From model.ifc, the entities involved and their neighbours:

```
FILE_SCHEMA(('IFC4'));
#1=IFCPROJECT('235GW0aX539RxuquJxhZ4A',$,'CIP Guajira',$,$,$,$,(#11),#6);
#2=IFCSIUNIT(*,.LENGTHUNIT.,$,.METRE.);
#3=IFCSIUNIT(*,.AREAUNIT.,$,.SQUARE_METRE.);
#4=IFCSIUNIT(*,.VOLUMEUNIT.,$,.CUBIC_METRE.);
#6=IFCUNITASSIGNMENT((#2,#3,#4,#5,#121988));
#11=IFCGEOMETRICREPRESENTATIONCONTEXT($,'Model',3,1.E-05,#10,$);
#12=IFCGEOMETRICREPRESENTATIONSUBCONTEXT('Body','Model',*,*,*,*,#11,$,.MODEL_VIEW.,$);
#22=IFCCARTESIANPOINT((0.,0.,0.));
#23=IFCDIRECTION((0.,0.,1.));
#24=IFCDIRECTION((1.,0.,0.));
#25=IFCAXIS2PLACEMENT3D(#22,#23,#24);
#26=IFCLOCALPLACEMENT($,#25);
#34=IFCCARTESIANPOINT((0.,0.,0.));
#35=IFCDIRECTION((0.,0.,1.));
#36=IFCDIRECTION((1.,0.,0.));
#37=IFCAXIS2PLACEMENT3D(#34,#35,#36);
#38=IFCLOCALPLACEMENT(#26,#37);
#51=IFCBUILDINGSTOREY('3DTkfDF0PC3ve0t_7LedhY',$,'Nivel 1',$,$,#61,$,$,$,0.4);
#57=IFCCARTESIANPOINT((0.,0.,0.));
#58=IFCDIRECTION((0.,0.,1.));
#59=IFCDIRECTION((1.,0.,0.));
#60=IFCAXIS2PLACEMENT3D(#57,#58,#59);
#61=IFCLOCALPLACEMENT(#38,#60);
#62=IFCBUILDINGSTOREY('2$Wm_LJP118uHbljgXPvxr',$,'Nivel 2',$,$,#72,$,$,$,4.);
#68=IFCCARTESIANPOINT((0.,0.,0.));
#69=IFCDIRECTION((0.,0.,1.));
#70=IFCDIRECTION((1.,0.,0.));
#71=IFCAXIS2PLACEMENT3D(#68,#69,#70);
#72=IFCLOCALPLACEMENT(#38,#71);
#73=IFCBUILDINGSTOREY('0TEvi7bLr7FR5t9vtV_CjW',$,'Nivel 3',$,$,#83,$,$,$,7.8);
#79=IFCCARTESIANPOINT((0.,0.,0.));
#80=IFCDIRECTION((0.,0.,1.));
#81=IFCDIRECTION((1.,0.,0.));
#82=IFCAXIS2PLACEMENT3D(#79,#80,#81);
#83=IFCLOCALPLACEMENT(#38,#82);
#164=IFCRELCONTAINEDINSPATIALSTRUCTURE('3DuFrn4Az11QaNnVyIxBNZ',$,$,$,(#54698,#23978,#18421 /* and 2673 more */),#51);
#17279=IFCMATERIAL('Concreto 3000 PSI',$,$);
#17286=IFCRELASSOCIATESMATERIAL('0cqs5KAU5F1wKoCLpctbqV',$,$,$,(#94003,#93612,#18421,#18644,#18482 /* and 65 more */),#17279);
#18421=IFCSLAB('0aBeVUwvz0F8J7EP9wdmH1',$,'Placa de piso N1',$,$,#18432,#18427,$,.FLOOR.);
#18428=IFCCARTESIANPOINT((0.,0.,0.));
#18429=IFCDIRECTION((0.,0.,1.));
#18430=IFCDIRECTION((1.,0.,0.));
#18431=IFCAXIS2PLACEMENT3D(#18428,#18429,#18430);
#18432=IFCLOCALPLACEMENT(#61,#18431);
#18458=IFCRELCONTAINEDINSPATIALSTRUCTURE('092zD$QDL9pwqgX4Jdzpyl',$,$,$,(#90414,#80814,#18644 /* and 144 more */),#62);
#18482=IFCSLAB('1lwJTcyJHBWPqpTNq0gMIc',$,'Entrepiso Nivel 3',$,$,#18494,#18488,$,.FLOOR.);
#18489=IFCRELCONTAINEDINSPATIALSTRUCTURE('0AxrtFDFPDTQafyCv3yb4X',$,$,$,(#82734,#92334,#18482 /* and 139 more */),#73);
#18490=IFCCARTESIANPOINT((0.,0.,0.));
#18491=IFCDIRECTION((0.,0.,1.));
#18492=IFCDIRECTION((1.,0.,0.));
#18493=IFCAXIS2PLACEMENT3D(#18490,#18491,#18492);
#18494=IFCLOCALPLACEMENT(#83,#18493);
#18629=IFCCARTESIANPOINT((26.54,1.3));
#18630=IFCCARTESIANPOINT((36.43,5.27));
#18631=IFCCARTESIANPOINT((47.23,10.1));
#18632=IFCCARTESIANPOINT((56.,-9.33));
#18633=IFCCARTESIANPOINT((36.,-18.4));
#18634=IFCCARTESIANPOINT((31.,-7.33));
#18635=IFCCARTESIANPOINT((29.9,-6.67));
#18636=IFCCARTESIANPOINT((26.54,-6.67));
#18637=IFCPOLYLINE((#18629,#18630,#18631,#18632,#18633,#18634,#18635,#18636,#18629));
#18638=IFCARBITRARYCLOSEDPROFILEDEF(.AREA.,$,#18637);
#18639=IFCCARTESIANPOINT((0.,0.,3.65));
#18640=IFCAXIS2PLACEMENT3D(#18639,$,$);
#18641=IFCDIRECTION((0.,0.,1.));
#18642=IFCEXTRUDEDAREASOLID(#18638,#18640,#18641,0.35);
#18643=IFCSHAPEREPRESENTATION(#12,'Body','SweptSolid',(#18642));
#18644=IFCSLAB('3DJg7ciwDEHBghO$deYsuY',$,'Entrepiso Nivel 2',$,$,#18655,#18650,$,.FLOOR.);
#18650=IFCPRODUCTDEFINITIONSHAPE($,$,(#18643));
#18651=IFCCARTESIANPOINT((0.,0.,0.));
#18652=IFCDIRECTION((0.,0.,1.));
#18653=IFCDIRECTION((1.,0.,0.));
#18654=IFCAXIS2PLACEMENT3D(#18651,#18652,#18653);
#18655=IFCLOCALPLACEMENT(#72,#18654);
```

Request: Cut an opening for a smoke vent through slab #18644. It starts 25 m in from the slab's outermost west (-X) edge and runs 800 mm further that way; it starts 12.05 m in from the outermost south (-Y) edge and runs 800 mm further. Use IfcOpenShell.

```python
import numpy as np
import ifcopenshell
import ifcopenshell.api.feature
import ifcopenshell.api.geometry
import ifcopenshell.api.root
import ifcopenshell.geom
import ifcopenshell.util.placement
import ifcopenshell.util.representation
import ifcopenshell.util.shape
import ifcopenshell.util.unit

model = ifcopenshell.open("model.ifc")
unit_scale = ifcopenshell.util.unit.calculate_unit_scale(model)
settings = ifcopenshell.geom.settings()


def volume(element):
    """Net volume in cubic metres, openings subtracted."""
    shape = ifcopenshell.geom.create_shape(settings, element)
    return ifcopenshell.util.shape.get_volume(shape.geometry)


slab = model.by_guid("3DJg7ciwDEHBghO$deYsuY")
before = volume(slab)

# Extent in the slab's own axes, in metres. The edges named are its -X and -Y sides.
slab_shape = ifcopenshell.geom.create_shape(settings, slab)
vertices = ifcopenshell.util.shape.get_vertices(slab_shape.geometry)
x_min, y_min, bottom = vertices.min(axis=0)
top = vertices[:, 2].max()

opening = ifcopenshell.api.root.create_entity(model, ifc_class="IfcOpeningElement", name="Smoke vent opening", predefined_type="OPENING")
context = ifcopenshell.util.representation.get_context(model, "Model", "Body", "MODEL_VIEW")
width, depth = 0.8, 0.8
outline = [(0.0, 0.0), (width, 0.0), (width, depth), (0.0, depth), (0.0, 0.0)]
# Overshoot both faces by 50 mm so the cut is clean.
shape = ifcopenshell.api.geometry.add_slab_representation(
    model, context=context, depth=top - bottom + 0.1, polyline=outline
)
ifcopenshell.api.geometry.assign_representation(model, product=opening, representation=shape)

matrix = ifcopenshell.util.placement.get_local_placement(slab.ObjectPlacement)
matrix[:, 3] = matrix @ np.append(np.array([x_min + 25, y_min + 12.05, bottom - 0.05]) / unit_scale, 1.0)
ifcopenshell.api.geometry.edit_object_placement(model, product=opening, matrix=matrix, is_si=False)
ifcopenshell.api.feature.add_feature(model, feature=opening, element=slab)

after = volume(slab)

print(f"slab volume {before:.3f} -> {after:.3f} m3")

model.write("model_edited.ifc")
```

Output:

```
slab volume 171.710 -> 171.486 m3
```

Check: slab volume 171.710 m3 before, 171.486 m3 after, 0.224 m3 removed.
